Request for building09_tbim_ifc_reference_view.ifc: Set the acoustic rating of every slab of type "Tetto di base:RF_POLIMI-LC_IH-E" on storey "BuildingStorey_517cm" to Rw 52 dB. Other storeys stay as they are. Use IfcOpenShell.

First a look at what the model holds.

```python
import ifcopenshell
import ifcopenshell.util.element

model = ifcopenshell.open("building09_tbim_ifc_reference_view.ifc")
print(model.schema)
storey = next(s for s in model.by_type("IfcBuildingStorey") if s.Name == "BuildingStorey_517cm")
slabs = [e for e in ifcopenshell.util.element.get_decomposition(storey) if e.is_a("IfcSlab")]
seen = {}
for e in slabs:
    element_type = ifcopenshell.util.element.get_type(e)
    key = (element_type.Name if element_type != e and element_type else None, ifcopenshell.util.element.get_pset(e, "Pset_SlabCommon", "AcousticRating"))
    seen[key] = seen.get(key, 0) + 1
for (name, value), count in sorted(seen.items(), key=str):
    print(count, "x", name, "|", value)
```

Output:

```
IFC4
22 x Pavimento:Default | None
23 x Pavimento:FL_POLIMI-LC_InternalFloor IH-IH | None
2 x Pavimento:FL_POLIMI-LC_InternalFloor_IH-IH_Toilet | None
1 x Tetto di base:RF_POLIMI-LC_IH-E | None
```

```python
import ifcopenshell
import ifcopenshell.api.pset
import ifcopenshell.util.element

model = ifcopenshell.open("building09_tbim_ifc_reference_view.ifc")

storey = next(s for s in model.by_type("IfcBuildingStorey") if s.Name == "BuildingStorey_517cm")
slabs = [e for e in ifcopenshell.util.element.get_decomposition(storey) if e.is_a("IfcSlab")]

count = 0
for e in slabs:
    element_type = ifcopenshell.util.element.get_type(e)
    if element_type in (None, e) or element_type.Name != "Tetto di base:RF_POLIMI-LC_IH-E":
        continue
    # add_pset returns the element's existing set when there is one.
    pset = ifcopenshell.api.pset.add_pset(model, product=e, name="Pset_SlabCommon")
    ifcopenshell.api.pset.edit_pset(model, pset=pset, properties={"AcousticRating": "Rw 52 dB"})
    count += 1

print(count, "slabs updated")

model.write("building09_tbim_ifc_reference_view-out.ifc")
```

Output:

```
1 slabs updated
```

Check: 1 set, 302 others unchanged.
